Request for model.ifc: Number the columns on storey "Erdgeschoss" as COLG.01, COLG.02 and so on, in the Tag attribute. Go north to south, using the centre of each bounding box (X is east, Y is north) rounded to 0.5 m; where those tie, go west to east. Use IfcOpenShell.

First a look at what the model holds.

```python
import ifcopenshell
import ifcopenshell.util.element
import ifcopenshell.util.placement

model = ifcopenshell.open("model.ifc")
print(model.schema)
storey = next(s for s in model.by_type("IfcBuildingStorey") if s.Name == "Erdgeschoss")
columns = [e for e in ifcopenshell.util.element.get_decomposition(storey) if e.is_a("IfcColumn")]
for e in sorted(columns, key=lambda e: e.id()):
    origin = ifcopenshell.util.placement.get_local_placement(e.ObjectPlacement)[:3, 3]
    print(e.id(), e.Tag, e.Name, origin.round(2) + 0.0, sep=" | ")
```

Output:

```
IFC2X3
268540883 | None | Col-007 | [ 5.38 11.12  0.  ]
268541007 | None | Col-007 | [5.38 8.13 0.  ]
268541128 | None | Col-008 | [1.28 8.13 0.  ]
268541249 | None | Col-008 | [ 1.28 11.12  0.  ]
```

```python
import ifcopenshell
import ifcopenshell.geom
import ifcopenshell.util.element
import ifcopenshell.util.shape

model = ifcopenshell.open("model.ifc")
settings = ifcopenshell.geom.settings()
settings.set("use-world-coords", True)


def centre(element):
    shape = ifcopenshell.geom.create_shape(settings, element)
    return ifcopenshell.util.shape.get_bbox_centroid(shape.geometry)


storey = next(s for s in model.by_type("IfcBuildingStorey") if s.Name == "Erdgeschoss")
columns = [e for e in ifcopenshell.util.element.get_decomposition(storey) if e.is_a("IfcColumn")]

# Insertion points can sit at a corner or the storey origin, so sort by the geometry (in metres).
centres = {e: centre(e) for e in columns}
columns.sort(key=lambda e: (-round(centres[e][1] / 0.5), centres[e][0]))

for i, e in enumerate(columns, start=1):
    number = f"COLG.{i:02d}"
    e.Tag = number
    print(e.id(), number)

model.write("model-out.ifc")
```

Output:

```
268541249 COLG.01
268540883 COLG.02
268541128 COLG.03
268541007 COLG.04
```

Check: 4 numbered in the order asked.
